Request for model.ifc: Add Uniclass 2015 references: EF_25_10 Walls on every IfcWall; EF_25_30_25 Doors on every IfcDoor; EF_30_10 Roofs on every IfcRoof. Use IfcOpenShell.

First a look at what the model holds.

```python
import ifcopenshell

model = ifcopenshell.open("model.ifc")
print(model.schema)
print("classifications:", [c.Name for c in model.by_type("IfcClassification")])
for ifc_class in ("IfcDoor", "IfcRoof", "IfcStair", "IfcWall", "IfcWindow"):
    print(ifc_class, len(model.by_type(ifc_class)))
```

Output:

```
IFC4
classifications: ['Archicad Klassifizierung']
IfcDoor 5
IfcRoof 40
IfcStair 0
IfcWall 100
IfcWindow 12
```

```python
import ifcopenshell
import ifcopenshell.api.classification

model = ifcopenshell.open("model.ifc")

system = ifcopenshell.api.classification.add_classification(model, classification="Uniclass 2015")

codes = {
    "IfcWall": ("EF_25_10", "Walls"),
    "IfcDoor": ("EF_25_30_25", "Doors"),
    "IfcRoof": ("EF_30_10", "Roofs"),
}
for ifc_class, (code, name) in codes.items():
    products = model.by_type(ifc_class)
    ifcopenshell.api.classification.add_reference(
        model, products=products, classification=system, identification=code, name=name
    )
    print(code, len(products))

model.write("model_rev.ifc")
```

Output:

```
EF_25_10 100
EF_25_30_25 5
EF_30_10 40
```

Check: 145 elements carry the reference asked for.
